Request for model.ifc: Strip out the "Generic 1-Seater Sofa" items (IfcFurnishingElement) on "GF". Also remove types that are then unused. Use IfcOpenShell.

First a look at what the model holds.

```python
import ifcopenshell
import ifcopenshell.util.element

model = ifcopenshell.open("model.ifc")
print(model.schema)
storey = next(s for s in model.by_type("IfcBuildingStorey") if s.Name == "GF")
furniture = [e for e in ifcopenshell.util.element.get_decomposition(storey) if e.is_a("IfcFurnishingElement")]
seen = {}
for e in furniture:
    element_type = ifcopenshell.util.element.get_type(e)
    name = element_type.Name if element_type not in (None, e) else None
    seen[name] = seen.get(name, 0) + 1
for name, count in sorted(seen.items(), key=str):
    print(count, "x", name)
```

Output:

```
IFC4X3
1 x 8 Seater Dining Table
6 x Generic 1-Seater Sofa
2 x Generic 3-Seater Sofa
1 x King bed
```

```python
import ifcopenshell
import ifcopenshell.api.root
import ifcopenshell.util.element

model = ifcopenshell.open("model.ifc")

storey = next(s for s in model.by_type("IfcBuildingStorey") if s.Name == "GF")
furniture = [e for e in ifcopenshell.util.element.get_decomposition(storey) if e.is_a("IfcFurnishingElement")]
targets = [e for e in furniture if (t := ifcopenshell.util.element.get_type(e)) not in (None, e) and t.Name == "Generic 1-Seater Sofa"]
types = {ifcopenshell.util.element.get_type(e) for e in targets} - {None, *targets}

for e in targets:
    ifcopenshell.api.root.remove_product(model, product=e)
print(len(targets), "removed")

unused = [t for t in types if not ifcopenshell.util.element.get_types(t)]
for t in unused:
    ifcopenshell.api.root.remove_product(model, product=t)
print(len(unused), "unused types removed")

model.write("model_edited.ifc")
```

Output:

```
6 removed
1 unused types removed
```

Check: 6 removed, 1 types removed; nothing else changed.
